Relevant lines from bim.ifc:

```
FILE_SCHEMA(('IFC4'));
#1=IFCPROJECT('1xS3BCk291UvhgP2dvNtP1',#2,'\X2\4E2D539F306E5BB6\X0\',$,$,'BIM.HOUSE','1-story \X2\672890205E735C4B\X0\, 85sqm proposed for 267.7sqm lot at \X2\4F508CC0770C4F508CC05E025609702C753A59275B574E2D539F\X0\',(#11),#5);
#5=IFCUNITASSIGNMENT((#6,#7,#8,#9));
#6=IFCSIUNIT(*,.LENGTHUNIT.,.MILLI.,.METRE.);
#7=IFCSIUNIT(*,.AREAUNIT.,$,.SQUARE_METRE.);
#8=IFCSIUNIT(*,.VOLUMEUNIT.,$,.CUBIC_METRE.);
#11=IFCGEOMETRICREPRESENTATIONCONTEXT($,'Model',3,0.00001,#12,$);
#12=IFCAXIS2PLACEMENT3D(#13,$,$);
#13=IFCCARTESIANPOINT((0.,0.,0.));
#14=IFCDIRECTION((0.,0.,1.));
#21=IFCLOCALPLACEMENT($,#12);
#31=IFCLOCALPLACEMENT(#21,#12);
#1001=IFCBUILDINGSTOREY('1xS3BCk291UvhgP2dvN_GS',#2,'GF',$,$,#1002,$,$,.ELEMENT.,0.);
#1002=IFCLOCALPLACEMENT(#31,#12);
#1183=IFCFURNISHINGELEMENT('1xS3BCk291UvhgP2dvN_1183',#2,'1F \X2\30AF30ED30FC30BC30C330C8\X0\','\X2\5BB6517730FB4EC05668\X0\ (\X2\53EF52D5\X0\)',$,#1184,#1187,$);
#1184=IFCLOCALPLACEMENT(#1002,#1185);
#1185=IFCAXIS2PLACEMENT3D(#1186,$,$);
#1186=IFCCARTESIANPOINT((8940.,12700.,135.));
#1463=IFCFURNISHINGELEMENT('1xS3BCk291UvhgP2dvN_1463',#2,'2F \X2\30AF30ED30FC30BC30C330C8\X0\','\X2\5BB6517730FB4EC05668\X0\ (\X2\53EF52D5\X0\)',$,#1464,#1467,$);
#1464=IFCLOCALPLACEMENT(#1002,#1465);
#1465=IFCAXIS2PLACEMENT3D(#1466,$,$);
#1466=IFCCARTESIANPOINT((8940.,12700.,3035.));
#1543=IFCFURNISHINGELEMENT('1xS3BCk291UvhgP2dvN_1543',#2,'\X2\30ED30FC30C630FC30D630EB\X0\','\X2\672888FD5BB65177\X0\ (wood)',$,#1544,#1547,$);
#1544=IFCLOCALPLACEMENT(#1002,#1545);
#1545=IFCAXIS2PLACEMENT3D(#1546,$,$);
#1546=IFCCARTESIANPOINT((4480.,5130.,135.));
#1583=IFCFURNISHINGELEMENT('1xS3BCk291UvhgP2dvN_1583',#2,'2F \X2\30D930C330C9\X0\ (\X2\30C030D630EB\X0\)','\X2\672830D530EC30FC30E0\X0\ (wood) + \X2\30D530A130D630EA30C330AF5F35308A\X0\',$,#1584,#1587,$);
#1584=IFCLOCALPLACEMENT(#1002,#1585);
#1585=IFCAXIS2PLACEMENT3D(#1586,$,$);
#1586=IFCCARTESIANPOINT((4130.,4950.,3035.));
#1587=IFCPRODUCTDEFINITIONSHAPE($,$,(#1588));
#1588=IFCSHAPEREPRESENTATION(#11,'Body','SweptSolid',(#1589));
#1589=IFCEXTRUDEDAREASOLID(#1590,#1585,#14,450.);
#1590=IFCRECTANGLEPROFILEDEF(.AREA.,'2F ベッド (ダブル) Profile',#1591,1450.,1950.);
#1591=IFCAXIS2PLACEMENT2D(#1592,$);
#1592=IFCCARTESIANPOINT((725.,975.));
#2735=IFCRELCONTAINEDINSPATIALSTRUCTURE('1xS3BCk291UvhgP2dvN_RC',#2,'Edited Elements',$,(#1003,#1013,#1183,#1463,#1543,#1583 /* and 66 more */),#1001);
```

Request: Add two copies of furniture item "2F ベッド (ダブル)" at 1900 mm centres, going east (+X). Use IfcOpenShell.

```python
import numpy as np
import ifcopenshell
import ifcopenshell.api.geometry
import ifcopenshell.api.root
import ifcopenshell.util.element
import ifcopenshell.util.placement

model = ifcopenshell.open("bim.ifc")


def reuse_history(source, copy):
    """copy_class also copies each property set's owner history, people and application; keep the originals."""
    for rel in copy.IsDefinedBy:
        if rel.is_a("IfcRelDefinesByProperties") and (history := rel.RelatingPropertyDefinition.OwnerHistory):
            rel.RelatingPropertyDefinition.OwnerHistory = source.OwnerHistory
            ifcopenshell.util.element.remove_deep2(model, history)


source = model.by_guid("1xS3BCk291UvhgP2dvN_1583")
base = ifcopenshell.util.placement.get_local_placement(source.ObjectPlacement)
step = np.array([1.0, 0.0, 0.0]) * 1900.0

for i in range(1, 3):
    copy = ifcopenshell.api.root.copy_class(model, product=source)
    copy.Representation = ifcopenshell.util.element.copy_deep(
        model, source.Representation, exclude=["IfcGeometricRepresentationContext", "IfcRepresentationMap"]
    )
    reuse_history(source, copy)
    matrix = base.copy()
    matrix[:3, 3] += i * step
    print("added at", matrix[:3, 3].round(3) + 0.0)
    ifcopenshell.api.geometry.edit_object_placement(model, product=copy, matrix=matrix, is_si=False)

model.write("bim-out.ifc")
```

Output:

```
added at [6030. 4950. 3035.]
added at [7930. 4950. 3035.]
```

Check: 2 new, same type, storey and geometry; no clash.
